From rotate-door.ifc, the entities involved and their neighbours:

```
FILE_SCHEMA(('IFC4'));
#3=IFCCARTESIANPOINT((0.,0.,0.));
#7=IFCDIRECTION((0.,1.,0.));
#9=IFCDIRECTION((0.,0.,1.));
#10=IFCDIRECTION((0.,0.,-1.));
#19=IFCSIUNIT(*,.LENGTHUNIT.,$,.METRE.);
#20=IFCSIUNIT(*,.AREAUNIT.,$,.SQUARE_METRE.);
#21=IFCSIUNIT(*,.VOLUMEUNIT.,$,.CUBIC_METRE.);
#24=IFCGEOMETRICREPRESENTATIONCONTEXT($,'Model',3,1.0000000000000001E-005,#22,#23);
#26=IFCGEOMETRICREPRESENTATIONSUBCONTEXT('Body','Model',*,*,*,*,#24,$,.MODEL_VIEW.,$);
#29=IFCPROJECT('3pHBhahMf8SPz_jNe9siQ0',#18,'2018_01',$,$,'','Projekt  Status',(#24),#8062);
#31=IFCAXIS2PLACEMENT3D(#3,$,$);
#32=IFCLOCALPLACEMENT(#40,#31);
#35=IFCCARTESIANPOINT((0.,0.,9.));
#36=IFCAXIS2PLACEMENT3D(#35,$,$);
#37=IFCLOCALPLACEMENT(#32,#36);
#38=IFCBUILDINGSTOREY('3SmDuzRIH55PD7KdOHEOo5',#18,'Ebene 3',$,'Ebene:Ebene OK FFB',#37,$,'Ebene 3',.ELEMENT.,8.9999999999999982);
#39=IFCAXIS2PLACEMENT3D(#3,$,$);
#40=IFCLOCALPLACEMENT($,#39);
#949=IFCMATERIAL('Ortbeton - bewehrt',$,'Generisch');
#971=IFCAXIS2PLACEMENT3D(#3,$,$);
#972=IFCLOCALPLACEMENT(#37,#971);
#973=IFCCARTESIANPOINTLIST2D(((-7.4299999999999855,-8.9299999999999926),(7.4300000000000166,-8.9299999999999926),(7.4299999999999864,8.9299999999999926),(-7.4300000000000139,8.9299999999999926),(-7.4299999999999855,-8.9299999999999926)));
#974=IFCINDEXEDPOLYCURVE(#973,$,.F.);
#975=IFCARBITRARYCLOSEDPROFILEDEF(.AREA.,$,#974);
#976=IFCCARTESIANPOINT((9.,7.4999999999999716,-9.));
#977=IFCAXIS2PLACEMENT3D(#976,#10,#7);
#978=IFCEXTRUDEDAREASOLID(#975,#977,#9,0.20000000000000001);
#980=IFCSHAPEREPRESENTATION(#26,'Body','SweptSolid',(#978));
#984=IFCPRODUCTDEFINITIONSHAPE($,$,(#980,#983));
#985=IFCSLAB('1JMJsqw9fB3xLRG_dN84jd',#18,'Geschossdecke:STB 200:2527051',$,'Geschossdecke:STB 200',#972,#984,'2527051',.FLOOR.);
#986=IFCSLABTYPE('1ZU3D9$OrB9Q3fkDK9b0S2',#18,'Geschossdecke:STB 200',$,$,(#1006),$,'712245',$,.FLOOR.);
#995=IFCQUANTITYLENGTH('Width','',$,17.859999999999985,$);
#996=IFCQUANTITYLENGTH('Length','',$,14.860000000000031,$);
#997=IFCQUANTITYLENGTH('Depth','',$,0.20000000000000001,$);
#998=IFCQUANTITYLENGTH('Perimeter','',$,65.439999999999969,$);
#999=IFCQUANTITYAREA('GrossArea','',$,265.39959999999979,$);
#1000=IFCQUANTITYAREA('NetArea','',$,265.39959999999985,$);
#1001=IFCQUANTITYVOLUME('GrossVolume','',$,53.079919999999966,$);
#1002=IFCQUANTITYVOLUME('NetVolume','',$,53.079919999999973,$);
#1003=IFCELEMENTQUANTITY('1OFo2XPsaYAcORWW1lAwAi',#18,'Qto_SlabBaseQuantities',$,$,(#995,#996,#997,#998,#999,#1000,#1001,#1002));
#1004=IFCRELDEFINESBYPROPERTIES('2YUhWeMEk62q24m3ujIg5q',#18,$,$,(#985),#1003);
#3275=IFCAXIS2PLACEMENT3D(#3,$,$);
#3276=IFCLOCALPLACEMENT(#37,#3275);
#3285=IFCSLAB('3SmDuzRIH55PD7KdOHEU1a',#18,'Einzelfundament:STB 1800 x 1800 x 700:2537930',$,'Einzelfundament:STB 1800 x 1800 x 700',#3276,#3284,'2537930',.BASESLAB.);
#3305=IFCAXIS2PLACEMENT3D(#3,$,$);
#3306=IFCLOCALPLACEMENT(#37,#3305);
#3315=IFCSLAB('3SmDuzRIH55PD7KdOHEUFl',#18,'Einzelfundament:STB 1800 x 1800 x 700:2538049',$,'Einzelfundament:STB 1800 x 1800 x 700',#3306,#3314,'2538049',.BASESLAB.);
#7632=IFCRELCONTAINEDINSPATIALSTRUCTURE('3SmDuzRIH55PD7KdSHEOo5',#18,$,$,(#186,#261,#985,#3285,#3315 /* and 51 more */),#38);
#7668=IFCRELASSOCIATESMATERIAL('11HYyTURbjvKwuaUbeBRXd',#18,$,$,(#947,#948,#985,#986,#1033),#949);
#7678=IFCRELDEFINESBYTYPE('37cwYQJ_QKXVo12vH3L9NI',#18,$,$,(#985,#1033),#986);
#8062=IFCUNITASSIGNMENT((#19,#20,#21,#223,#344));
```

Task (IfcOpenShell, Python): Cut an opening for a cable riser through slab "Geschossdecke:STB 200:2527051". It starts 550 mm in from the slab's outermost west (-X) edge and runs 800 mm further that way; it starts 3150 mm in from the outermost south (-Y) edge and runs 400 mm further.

```python
import numpy as np
import ifcopenshell
import ifcopenshell.api.feature
import ifcopenshell.api.geometry
import ifcopenshell.api.pset
import ifcopenshell.api.root
import ifcopenshell.geom
import ifcopenshell.util.element
import ifcopenshell.util.placement
import ifcopenshell.util.representation
import ifcopenshell.util.shape
import ifcopenshell.util.unit

model = ifcopenshell.open("rotate-door.ifc")
unit_scale = ifcopenshell.util.unit.calculate_unit_scale(model)
area_scale = ifcopenshell.util.unit.calculate_unit_scale(model, "AREAUNIT")
volume_scale = ifcopenshell.util.unit.calculate_unit_scale(model, "VOLUMEUNIT")
settings = ifcopenshell.geom.settings()


def volume(element):
    """Net volume in cubic metres, openings subtracted."""
    shape = ifcopenshell.geom.create_shape(settings, element)
    return ifcopenshell.util.shape.get_volume(shape.geometry)


slab = model.by_guid("1JMJsqw9fB3xLRG_dN84jd")
before = volume(slab)

# Extent in the slab's own axes, in metres. The edges named are its -X and -Y sides.
slab_shape = ifcopenshell.geom.create_shape(settings, slab)
vertices = ifcopenshell.util.shape.get_vertices(slab_shape.geometry)
x_min, y_min, bottom = vertices.min(axis=0)
top = vertices[:, 2].max()

opening = ifcopenshell.api.root.create_entity(model, ifc_class="IfcOpeningElement", name="Cable riser opening", predefined_type="OPENING")
context = ifcopenshell.util.representation.get_context(model, "Model", "Body", "MODEL_VIEW")
width, depth = 0.8, 0.4
outline = [(0.0, 0.0), (width, 0.0), (width, depth), (0.0, depth), (0.0, 0.0)]
# Overshoot both faces by 50 mm so the cut is clean.
shape = ifcopenshell.api.geometry.add_slab_representation(
    model, context=context, depth=top - bottom + 0.1, polyline=outline
)
ifcopenshell.api.geometry.assign_representation(model, product=opening, representation=shape)

matrix = ifcopenshell.util.placement.get_local_placement(slab.ObjectPlacement)
matrix[:, 3] = matrix @ np.append(np.array([x_min + 0.55, y_min + 3.15, bottom - 0.05]) / unit_scale, 1.0)
ifcopenshell.api.geometry.edit_object_placement(model, product=opening, matrix=matrix, is_si=False)
ifcopenshell.api.feature.add_feature(model, feature=opening, element=slab)

after = volume(slab)

# Update the slab's stored quantities.
qto = model.by_id(ifcopenshell.util.element.get_pset(slab, "Qto_SlabBaseQuantities", should_inherit=False)["id"])
ifcopenshell.api.pset.edit_qto(model, qto=qto, properties={
    "NetArea": after / (top - bottom) / area_scale,
    "NetVolume": after / volume_scale,
})

print(f"slab volume {before:.3f} -> {after:.3f} m3")

model.write("rotate-door_edited.ifc")
```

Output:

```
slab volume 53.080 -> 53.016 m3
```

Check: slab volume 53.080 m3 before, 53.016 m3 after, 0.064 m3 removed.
